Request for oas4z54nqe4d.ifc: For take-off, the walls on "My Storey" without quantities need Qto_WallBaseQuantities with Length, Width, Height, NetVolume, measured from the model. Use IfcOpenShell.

First a look at what the model holds.

```python
import ifcopenshell
import ifcopenshell.util.element
import ifcopenshell.util.unit

model = ifcopenshell.open("oas4z54nqe4d.ifc")
print(model.schema)
for unit_type in ("LENGTHUNIT", "AREAUNIT", "VOLUMEUNIT"):
    print(unit_type, ifcopenshell.util.unit.calculate_unit_scale(model, unit_type))
storey = next(s for s in model.by_type("IfcBuildingStorey") if s.Name == "My Storey")
walls = [e for e in ifcopenshell.util.element.get_decomposition(storey) if e.is_a("IfcWall")]
for e in sorted(walls, key=lambda e: e.id()):
    print(e.id(), e.is_a(), e.Name, list(ifcopenshell.util.element.get_psets(e, qtos_only=True)), sep=" | ")
```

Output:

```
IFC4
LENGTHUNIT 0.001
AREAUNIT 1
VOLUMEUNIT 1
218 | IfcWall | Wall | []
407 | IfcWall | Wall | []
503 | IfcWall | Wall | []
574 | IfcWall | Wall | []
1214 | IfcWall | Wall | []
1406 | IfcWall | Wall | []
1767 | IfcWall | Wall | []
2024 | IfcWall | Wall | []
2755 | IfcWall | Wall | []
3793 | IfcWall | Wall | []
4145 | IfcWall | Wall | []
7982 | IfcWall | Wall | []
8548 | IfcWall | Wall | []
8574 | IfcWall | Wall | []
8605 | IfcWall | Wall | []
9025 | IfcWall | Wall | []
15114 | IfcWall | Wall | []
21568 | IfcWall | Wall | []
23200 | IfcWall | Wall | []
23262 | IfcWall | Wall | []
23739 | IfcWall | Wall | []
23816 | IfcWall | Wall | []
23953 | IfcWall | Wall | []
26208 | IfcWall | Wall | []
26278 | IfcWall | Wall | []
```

```python
import ifcopenshell
import ifcopenshell.api.pset
import ifcopenshell.geom
import ifcopenshell.util.element
import ifcopenshell.util.shape
import ifcopenshell.util.unit

model = ifcopenshell.open("oas4z54nqe4d.ifc")
unit_scale = ifcopenshell.util.unit.calculate_unit_scale(model)
volume_scale = ifcopenshell.util.unit.calculate_unit_scale(model, "VOLUMEUNIT")
settings = ifcopenshell.geom.settings()

storey = next(s for s in model.by_type("IfcBuildingStorey") if s.Name == "My Storey")
walls = [e for e in ifcopenshell.util.element.get_decomposition(storey) if e.is_a("IfcWall")]

for e in sorted(walls, key=lambda e: e.id()):
    if ifcopenshell.util.element.get_psets(e, qtos_only=True, should_inherit=False):
        continue
    # Geometry comes back in metres, in the element's own axes.
    shape = ifcopenshell.geom.create_shape(settings, e)
    values = {
        "Length": ifcopenshell.util.shape.get_x(shape.geometry) / unit_scale,
        "Width": ifcopenshell.util.shape.get_y(shape.geometry) / unit_scale,
        "Height": ifcopenshell.util.shape.get_z(shape.geometry) / unit_scale,
        "NetVolume": ifcopenshell.util.shape.get_volume(shape.geometry) / volume_scale,
    }
    qto = ifcopenshell.api.pset.add_qto(model, product=e, name="Qto_WallBaseQuantities")
    ifcopenshell.api.pset.edit_qto(model, qto=qto, properties=values)
    print(e.id(), {k: round(v, 3) for k, v in values.items()})

model.write("oas4z54nqe4d_updated.ifc")
```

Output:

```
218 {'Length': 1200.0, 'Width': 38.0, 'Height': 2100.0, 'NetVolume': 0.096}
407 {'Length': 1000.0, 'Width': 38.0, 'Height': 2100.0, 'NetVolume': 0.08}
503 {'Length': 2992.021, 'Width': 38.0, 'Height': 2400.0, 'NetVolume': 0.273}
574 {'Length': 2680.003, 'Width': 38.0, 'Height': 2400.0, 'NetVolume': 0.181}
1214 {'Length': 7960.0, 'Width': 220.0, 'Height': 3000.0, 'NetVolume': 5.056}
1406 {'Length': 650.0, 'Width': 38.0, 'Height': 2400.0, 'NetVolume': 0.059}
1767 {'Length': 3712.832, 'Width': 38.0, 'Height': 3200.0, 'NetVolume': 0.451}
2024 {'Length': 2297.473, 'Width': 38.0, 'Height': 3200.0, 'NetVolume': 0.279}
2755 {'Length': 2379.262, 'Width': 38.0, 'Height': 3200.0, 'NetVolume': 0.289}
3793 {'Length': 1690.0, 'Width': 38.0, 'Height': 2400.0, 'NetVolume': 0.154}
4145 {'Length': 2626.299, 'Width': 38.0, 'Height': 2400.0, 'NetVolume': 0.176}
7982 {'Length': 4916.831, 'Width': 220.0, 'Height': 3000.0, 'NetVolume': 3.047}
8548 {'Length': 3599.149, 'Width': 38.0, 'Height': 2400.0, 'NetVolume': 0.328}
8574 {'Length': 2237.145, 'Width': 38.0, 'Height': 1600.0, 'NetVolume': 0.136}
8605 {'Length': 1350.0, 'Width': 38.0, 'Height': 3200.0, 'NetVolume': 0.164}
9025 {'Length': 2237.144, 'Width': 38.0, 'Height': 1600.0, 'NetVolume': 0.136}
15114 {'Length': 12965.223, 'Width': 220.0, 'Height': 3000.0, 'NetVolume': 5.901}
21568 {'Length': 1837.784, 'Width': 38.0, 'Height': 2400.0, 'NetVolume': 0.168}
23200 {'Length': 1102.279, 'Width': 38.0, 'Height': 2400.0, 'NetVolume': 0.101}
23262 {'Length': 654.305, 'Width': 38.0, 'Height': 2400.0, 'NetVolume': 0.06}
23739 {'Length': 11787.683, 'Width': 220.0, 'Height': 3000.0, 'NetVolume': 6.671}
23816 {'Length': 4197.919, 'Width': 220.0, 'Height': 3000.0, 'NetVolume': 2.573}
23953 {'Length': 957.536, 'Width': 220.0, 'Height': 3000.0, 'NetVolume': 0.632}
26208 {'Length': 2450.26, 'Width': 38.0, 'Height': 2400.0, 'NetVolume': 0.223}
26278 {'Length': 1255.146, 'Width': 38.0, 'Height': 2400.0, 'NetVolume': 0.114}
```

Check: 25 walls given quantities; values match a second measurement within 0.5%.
